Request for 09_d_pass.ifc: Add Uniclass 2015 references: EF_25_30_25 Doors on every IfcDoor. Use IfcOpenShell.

First a look at what the model holds.

```python
import ifcopenshell

model = ifcopenshell.open("09_d_pass.ifc")
print(model.schema)
print("classifications:", [c.Name for c in model.by_type("IfcClassification")])
for ifc_class in ("IfcDoor", "IfcRoof", "IfcStair", "IfcWall", "IfcWindow"):
    print(ifc_class, len(model.by_type(ifc_class)))
```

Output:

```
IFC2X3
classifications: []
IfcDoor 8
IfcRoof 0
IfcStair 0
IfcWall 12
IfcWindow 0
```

```python
import ifcopenshell
import ifcopenshell.api.classification

model = ifcopenshell.open("09_d_pass.ifc")

# IFC2X3 requires Source and Edition and has no link from the project to the system.
system = model.create_entity("IfcClassification", Source="NBS", Edition="2015", Name="Uniclass 2015")

codes = {
    "IfcDoor": ("EF_25_30_25", "Doors"),
}
for ifc_class, (code, name) in codes.items():
    products = model.by_type(ifc_class)
    ifcopenshell.api.classification.add_reference(
        model, products=products, classification=system, identification=code, name=name
    )
    print(code, len(products))

model.write("09_d_pass_rev.ifc")
```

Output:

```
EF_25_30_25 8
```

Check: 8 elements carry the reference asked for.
